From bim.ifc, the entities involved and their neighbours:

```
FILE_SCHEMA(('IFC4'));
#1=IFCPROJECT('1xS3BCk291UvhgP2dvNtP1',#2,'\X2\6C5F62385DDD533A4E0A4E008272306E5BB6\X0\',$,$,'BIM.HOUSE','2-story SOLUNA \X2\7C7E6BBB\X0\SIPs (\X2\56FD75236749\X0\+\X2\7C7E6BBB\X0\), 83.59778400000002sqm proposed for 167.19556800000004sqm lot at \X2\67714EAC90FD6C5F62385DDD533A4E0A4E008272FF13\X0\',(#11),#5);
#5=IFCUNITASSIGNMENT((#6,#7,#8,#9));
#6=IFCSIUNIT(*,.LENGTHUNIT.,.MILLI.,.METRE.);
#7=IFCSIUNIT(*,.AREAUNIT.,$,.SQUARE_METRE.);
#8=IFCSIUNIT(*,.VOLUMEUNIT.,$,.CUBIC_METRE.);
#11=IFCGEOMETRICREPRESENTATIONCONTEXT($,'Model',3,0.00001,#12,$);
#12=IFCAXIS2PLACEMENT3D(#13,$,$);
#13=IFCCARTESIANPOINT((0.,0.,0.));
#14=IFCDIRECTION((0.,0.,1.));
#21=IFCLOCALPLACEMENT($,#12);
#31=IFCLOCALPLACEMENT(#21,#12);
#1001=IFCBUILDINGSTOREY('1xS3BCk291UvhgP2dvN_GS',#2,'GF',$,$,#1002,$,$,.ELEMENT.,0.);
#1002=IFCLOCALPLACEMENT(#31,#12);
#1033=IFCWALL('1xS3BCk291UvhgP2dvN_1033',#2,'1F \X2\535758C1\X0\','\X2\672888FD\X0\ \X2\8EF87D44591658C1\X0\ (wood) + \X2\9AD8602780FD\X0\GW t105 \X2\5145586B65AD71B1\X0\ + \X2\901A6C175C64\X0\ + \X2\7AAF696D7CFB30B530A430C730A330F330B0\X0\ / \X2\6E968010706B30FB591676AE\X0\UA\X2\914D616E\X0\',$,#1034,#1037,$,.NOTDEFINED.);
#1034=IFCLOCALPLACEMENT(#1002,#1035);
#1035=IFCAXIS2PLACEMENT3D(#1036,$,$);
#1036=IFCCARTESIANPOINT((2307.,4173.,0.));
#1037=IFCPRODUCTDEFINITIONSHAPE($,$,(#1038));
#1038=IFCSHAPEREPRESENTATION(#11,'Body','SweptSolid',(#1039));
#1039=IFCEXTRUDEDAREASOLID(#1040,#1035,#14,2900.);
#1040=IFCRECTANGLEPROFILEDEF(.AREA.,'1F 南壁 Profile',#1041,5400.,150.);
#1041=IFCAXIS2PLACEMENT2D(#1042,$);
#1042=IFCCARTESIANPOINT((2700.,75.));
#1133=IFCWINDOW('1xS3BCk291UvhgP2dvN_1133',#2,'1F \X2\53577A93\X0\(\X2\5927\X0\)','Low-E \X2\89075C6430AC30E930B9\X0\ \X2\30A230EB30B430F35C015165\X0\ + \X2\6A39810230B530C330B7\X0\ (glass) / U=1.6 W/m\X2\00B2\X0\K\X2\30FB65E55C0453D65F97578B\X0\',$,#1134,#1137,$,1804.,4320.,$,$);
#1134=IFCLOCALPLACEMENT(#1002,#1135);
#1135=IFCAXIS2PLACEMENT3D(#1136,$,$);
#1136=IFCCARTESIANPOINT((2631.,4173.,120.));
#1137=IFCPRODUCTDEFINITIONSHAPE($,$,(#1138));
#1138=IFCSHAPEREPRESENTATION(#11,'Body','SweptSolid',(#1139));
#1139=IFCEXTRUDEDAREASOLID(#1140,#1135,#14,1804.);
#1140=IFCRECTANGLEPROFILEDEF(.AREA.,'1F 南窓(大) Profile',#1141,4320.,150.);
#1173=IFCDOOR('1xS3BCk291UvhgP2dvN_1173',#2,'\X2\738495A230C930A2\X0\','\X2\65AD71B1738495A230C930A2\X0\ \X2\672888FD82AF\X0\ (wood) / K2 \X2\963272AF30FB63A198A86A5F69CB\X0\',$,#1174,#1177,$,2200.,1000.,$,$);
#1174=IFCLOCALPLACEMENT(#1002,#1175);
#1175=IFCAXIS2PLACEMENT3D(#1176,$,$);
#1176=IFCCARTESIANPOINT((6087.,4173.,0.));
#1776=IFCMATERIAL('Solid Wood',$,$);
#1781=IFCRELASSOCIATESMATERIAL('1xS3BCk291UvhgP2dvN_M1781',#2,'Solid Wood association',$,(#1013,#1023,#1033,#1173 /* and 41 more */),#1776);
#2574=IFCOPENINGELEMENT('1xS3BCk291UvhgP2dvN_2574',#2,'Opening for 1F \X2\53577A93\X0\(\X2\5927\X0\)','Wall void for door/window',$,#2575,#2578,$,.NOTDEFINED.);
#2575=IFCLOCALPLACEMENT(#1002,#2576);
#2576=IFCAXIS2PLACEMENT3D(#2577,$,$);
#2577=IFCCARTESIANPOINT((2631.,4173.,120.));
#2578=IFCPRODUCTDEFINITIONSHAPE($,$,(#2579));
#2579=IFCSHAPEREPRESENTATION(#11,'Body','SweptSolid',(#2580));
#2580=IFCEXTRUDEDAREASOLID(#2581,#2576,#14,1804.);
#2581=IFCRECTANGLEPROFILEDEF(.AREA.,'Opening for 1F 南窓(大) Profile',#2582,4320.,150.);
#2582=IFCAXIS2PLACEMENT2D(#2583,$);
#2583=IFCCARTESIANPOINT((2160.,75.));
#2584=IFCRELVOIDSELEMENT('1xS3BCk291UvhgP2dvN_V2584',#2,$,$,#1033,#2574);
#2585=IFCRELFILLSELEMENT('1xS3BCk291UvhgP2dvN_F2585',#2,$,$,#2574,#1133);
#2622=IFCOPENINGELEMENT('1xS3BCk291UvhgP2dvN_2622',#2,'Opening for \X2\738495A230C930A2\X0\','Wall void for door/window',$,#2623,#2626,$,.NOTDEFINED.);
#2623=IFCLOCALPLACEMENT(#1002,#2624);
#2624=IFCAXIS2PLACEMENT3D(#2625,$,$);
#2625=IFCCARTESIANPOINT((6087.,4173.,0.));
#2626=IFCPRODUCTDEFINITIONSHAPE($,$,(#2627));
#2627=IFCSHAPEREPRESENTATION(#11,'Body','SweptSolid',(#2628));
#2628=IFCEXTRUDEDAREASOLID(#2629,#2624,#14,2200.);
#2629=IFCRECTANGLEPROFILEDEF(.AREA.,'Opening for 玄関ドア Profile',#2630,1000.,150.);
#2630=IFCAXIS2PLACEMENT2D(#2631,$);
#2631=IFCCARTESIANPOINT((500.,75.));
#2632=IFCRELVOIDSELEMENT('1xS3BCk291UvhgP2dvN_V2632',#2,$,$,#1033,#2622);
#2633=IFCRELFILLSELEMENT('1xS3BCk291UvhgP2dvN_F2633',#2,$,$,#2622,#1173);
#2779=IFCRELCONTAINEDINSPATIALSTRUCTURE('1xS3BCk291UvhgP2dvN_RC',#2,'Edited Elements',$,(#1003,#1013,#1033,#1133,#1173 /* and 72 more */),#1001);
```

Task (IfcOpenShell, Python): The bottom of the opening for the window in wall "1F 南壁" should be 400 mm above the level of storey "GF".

```python
import numpy as np
import ifcopenshell
import ifcopenshell.api.geometry
import ifcopenshell.geom
import ifcopenshell.util.element
import ifcopenshell.util.placement
import ifcopenshell.util.shape
import ifcopenshell.util.unit

model = ifcopenshell.open("bim.ifc")
unit_scale = ifcopenshell.util.unit.calculate_unit_scale(model)

window = model.by_guid("1xS3BCk291UvhgP2dvN_1133")
opening = window.FillsVoids[0].RelatingOpeningElement
storey = ifcopenshell.util.element.get_container(window, ifc_class="IfcBuildingStorey")
level = ifcopenshell.util.placement.get_local_placement(storey.ObjectPlacement)[2, 3]

# The opening's origin need not be at the sill, so measure its lowest point.
shape = ifcopenshell.geom.create_shape(ifcopenshell.geom.settings(), opening)
bottom = ifcopenshell.util.shape.get_shape_bottom_elevation(shape, shape.geometry) / unit_scale
dz = level + 400.0 - bottom

shift = np.array([0.0, 0.0, dz])
# The window is not placed relative to its opening, so move both.
for product in (opening, window):
    matrix = ifcopenshell.util.placement.get_local_placement(product.ObjectPlacement)
    matrix[:3, 3] += shift
    ifcopenshell.api.geometry.edit_object_placement(model, product=product, matrix=matrix, is_si=False)

print(f"moved by {dz * unit_scale:+.3f} m")

model.write("bim-out.ifc")
```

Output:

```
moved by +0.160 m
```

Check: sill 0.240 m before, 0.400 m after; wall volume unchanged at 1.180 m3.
